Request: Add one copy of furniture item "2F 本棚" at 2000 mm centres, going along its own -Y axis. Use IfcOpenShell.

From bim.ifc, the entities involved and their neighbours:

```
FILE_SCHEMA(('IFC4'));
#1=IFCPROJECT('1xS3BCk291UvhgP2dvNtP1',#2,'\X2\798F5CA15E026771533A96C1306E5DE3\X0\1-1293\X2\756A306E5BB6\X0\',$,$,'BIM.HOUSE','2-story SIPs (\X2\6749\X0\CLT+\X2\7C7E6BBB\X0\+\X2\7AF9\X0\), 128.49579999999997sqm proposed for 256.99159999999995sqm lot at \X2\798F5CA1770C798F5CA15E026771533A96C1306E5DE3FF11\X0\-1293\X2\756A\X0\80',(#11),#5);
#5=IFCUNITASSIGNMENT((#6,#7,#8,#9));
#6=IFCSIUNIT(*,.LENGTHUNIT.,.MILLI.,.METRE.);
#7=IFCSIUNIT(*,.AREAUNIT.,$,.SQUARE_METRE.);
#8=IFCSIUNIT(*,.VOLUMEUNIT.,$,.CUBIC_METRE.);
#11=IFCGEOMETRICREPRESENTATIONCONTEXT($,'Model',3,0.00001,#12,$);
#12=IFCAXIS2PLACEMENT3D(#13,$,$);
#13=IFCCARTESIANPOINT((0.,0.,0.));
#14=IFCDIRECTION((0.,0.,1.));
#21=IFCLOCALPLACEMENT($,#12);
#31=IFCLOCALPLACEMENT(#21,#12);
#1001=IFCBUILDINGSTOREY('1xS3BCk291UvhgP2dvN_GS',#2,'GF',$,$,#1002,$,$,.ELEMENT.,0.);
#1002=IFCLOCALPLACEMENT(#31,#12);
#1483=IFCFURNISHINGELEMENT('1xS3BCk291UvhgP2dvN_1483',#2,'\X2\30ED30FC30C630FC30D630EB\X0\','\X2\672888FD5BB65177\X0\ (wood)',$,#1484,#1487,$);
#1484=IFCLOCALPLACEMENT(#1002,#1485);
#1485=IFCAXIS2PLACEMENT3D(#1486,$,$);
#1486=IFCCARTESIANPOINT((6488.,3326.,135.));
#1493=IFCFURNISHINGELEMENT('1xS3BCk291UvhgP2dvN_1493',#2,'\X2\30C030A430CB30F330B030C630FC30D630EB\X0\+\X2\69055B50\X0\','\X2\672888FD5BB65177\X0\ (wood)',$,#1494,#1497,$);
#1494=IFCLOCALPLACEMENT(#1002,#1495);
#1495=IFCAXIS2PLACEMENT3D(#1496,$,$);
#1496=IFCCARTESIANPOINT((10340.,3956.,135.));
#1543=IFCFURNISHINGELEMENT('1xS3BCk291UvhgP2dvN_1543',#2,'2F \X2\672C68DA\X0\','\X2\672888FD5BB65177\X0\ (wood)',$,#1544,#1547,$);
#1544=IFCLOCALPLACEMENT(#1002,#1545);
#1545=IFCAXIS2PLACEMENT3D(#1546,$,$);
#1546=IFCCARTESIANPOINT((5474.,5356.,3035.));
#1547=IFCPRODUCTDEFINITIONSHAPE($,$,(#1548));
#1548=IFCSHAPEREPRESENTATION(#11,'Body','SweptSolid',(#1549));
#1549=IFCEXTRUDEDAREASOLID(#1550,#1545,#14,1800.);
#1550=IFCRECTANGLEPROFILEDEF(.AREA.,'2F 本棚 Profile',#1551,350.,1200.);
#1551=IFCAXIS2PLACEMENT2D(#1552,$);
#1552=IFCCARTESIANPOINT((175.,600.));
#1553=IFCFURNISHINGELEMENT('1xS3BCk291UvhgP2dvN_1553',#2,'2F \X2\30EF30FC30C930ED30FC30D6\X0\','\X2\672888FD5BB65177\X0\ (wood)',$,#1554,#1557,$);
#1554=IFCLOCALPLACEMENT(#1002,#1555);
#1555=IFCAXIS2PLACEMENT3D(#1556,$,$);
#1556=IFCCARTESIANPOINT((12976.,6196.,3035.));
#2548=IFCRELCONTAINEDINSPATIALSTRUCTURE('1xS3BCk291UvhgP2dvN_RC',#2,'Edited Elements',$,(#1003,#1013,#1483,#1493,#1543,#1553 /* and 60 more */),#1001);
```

```python
import ifcopenshell
import ifcopenshell.api.geometry
import ifcopenshell.api.root
import ifcopenshell.util.element
import ifcopenshell.util.placement

model = ifcopenshell.open("bim.ifc")


def reuse_history(source, copy):
    """copy_class also copies each property set's owner history, people and application; keep the originals."""
    for rel in copy.IsDefinedBy:
        if rel.is_a("IfcRelDefinesByProperties") and (history := rel.RelatingPropertyDefinition.OwnerHistory):
            rel.RelatingPropertyDefinition.OwnerHistory = source.OwnerHistory
            ifcopenshell.util.element.remove_deep2(model, history)


source = model.by_guid("1xS3BCk291UvhgP2dvN_1543")
base = ifcopenshell.util.placement.get_local_placement(source.ObjectPlacement)
step = -base[:3, 1] * 2000.0

for i in range(1, 2):
    copy = ifcopenshell.api.root.copy_class(model, product=source)
    copy.Representation = ifcopenshell.util.element.copy_deep(
        model, source.Representation, exclude=["IfcGeometricRepresentationContext", "IfcRepresentationMap"]
    )
    reuse_history(source, copy)
    matrix = base.copy()
    matrix[:3, 3] += i * step
    print("added at", matrix[:3, 3].round(3) + 0.0)
    ifcopenshell.api.geometry.edit_object_placement(model, product=copy, matrix=matrix, is_si=False)

model.write("bim_rev.ifc")
```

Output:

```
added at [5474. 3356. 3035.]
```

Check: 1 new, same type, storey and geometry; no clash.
